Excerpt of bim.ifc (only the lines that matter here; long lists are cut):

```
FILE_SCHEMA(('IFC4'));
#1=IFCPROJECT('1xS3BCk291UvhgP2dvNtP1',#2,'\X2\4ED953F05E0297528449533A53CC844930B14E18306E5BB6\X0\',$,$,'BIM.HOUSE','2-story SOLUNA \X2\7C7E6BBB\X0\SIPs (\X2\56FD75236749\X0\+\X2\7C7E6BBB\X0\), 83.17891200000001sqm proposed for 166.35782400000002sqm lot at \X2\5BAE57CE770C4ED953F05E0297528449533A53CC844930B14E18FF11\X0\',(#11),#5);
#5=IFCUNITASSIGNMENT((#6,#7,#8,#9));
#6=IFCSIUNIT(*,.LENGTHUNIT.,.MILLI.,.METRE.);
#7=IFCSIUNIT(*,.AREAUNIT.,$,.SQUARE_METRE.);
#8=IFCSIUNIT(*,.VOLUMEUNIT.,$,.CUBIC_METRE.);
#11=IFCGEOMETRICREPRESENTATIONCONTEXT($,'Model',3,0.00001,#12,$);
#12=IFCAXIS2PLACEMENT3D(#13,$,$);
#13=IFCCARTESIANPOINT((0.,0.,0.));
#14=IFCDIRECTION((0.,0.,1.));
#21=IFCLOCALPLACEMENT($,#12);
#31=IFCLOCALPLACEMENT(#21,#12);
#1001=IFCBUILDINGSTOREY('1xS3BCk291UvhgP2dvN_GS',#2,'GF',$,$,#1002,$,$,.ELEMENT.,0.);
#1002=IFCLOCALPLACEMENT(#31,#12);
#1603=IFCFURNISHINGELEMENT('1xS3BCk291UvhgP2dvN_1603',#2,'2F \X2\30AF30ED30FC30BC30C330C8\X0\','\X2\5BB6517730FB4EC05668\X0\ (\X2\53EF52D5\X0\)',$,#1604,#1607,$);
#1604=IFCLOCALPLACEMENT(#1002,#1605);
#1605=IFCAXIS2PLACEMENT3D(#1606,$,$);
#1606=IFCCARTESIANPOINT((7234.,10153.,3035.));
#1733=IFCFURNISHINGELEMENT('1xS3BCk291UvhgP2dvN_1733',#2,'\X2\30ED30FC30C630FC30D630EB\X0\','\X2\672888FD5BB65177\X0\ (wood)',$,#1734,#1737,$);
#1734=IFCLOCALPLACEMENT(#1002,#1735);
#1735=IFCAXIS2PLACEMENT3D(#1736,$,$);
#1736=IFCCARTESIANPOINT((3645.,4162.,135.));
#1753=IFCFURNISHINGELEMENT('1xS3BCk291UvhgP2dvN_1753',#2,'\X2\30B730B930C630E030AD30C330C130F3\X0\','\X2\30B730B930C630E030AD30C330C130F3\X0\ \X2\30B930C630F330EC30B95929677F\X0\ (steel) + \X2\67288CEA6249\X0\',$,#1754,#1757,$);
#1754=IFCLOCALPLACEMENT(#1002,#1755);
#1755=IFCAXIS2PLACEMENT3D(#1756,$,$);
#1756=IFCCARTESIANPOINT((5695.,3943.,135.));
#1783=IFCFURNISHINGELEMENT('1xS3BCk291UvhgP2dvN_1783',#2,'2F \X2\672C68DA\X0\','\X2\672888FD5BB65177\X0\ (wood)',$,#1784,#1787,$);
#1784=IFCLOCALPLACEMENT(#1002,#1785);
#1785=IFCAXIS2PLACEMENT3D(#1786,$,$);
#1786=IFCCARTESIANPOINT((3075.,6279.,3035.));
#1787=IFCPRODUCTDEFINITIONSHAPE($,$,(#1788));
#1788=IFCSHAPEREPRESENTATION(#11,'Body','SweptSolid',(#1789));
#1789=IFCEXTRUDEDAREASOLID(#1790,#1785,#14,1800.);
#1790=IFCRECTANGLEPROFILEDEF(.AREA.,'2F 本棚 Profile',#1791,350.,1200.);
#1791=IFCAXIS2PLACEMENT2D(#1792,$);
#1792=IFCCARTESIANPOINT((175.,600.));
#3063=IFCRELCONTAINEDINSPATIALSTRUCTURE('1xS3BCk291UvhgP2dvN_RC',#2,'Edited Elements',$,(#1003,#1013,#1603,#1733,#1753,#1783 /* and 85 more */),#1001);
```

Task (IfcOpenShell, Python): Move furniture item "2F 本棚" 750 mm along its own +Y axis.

```python
import ifcopenshell
import ifcopenshell.api.geometry
import ifcopenshell.util.placement
import ifcopenshell.util.unit

model = ifcopenshell.open("bim.ifc")
unit_scale = ifcopenshell.util.unit.calculate_unit_scale(model)

item = model.by_guid("1xS3BCk291UvhgP2dvN_1783")
matrix = ifcopenshell.util.placement.get_local_placement(item.ObjectPlacement)
matrix[:3, 3] += matrix[:3, 1] * 0.75 / unit_scale
ifcopenshell.api.geometry.edit_object_placement(model, product=item, matrix=matrix, is_si=False)

print(ifcopenshell.util.placement.get_local_placement(item.ObjectPlacement).round(3) + 0.0)

model.write("bim_v2.ifc")
```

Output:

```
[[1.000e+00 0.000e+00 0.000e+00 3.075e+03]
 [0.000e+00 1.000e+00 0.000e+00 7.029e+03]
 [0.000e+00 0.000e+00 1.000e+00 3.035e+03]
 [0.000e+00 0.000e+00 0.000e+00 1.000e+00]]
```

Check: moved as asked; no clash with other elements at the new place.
